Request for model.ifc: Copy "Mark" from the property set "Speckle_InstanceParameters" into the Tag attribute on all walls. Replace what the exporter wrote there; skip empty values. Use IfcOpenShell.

First a look at what the model holds.

```python
import ifcopenshell
import ifcopenshell.util.element

model = ifcopenshell.open("model.ifc")
print(model.schema)
walls = model.by_type("IfcWall")
print(len(walls), "walls")
for e in walls[:8]:
    source = ifcopenshell.util.element.get_pset(e, "Speckle_InstanceParameters", "Mark")
    target = e.Tag
    print(e.id(), repr(source), repr(target), sep=" | ")
```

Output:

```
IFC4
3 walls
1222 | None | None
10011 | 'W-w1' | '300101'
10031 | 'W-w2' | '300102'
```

```python
import ifcopenshell
import ifcopenshell.util.element

model = ifcopenshell.open("model.ifc")

count = 0
for e in model.by_type("IfcWall"):
    value = ifcopenshell.util.element.get_pset(e, "Speckle_InstanceParameters", "Mark")
    current = e.Tag
    if not value or not value.strip() or current == value:
        continue
    e.Tag = value
    count += 1

print(count, "walls updated")

model.write("model_edited.ifc")
```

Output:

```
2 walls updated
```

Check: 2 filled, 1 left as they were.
